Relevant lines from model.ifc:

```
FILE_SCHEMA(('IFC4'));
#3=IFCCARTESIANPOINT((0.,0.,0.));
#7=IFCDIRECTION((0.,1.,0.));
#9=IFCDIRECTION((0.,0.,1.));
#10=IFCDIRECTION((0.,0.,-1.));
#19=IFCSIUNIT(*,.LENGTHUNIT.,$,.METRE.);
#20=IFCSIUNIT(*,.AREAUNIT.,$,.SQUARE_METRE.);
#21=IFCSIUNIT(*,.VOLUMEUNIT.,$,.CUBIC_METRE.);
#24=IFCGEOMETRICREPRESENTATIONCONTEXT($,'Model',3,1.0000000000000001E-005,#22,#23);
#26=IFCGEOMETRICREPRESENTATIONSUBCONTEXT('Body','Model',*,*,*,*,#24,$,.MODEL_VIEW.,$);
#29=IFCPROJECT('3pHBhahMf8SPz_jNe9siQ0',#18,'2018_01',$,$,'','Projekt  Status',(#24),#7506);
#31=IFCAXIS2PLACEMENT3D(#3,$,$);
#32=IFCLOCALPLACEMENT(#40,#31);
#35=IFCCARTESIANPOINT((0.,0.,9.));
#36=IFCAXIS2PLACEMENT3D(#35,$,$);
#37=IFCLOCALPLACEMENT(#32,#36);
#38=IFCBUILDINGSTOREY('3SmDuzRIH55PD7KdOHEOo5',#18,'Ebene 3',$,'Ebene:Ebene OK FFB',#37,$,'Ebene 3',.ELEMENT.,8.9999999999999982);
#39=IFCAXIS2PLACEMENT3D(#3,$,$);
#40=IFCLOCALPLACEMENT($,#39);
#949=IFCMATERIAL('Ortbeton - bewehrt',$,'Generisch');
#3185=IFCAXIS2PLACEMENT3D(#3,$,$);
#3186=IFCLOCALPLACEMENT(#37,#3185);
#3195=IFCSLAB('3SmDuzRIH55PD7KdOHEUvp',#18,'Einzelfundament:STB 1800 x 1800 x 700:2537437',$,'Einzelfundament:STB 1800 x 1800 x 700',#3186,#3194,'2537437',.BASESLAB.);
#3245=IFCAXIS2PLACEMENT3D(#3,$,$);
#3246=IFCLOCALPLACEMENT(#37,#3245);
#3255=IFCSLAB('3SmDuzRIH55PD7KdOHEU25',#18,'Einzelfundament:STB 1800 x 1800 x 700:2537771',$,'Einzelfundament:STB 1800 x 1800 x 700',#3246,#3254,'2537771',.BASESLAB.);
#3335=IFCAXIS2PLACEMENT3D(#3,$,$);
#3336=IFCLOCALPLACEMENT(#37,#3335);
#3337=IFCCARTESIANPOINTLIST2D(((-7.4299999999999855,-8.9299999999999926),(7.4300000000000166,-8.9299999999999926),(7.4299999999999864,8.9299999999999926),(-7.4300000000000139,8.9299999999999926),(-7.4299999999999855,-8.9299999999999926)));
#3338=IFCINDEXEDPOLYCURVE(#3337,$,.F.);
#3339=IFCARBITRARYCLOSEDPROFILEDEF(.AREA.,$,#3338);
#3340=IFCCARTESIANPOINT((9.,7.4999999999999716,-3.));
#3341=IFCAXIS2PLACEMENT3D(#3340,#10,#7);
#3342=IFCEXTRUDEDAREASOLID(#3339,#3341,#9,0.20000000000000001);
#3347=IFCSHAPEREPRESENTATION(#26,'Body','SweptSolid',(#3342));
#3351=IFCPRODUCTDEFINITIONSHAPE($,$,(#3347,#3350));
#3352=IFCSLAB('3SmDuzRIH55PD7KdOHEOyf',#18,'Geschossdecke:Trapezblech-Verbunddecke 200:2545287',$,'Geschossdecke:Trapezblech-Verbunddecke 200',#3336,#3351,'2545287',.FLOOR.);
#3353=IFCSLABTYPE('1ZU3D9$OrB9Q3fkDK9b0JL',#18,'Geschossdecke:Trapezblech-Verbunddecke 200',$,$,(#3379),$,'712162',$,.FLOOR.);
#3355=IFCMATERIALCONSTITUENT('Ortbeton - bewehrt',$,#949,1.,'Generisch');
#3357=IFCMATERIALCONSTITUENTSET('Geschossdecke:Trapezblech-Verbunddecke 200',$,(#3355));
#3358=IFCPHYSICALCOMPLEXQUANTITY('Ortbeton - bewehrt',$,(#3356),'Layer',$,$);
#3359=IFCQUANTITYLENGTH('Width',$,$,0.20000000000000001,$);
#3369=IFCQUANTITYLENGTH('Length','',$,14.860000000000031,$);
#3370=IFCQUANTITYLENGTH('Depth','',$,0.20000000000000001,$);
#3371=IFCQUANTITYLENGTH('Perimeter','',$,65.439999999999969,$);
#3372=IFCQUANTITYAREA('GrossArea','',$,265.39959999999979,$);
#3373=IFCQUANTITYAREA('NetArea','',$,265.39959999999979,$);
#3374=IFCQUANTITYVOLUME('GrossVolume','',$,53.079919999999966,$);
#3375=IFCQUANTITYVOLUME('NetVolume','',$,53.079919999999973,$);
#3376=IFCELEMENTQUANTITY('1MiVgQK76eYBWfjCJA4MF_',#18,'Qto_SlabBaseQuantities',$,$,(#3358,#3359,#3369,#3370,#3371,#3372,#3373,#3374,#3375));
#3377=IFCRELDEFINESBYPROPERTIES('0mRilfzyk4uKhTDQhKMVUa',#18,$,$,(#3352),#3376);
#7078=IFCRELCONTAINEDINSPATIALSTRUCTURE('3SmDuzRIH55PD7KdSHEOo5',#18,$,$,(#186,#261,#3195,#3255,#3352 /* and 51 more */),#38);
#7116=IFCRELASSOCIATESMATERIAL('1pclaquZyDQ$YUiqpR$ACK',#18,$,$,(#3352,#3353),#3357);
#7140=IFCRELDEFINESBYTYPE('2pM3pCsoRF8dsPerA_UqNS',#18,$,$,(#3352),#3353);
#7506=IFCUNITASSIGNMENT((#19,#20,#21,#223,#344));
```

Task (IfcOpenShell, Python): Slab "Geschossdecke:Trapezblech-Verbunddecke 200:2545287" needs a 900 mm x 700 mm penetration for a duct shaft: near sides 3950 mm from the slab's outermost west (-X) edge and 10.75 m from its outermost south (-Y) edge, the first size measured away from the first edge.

```python
import numpy as np
import ifcopenshell
import ifcopenshell.api.feature
import ifcopenshell.api.geometry
import ifcopenshell.api.pset
import ifcopenshell.api.root
import ifcopenshell.geom
import ifcopenshell.util.element
import ifcopenshell.util.placement
import ifcopenshell.util.representation
import ifcopenshell.util.shape
import ifcopenshell.util.unit

model = ifcopenshell.open("model.ifc")
unit_scale = ifcopenshell.util.unit.calculate_unit_scale(model)
area_scale = ifcopenshell.util.unit.calculate_unit_scale(model, "AREAUNIT")
volume_scale = ifcopenshell.util.unit.calculate_unit_scale(model, "VOLUMEUNIT")
settings = ifcopenshell.geom.settings()


def volume(element):
    """Net volume in cubic metres, openings subtracted."""
    shape = ifcopenshell.geom.create_shape(settings, element)
    return ifcopenshell.util.shape.get_volume(shape.geometry)


slab = model.by_guid("3SmDuzRIH55PD7KdOHEOyf")
before = volume(slab)

# Extent in the slab's own axes, in metres. The edges named are its -X and -Y sides.
slab_shape = ifcopenshell.geom.create_shape(settings, slab)
vertices = ifcopenshell.util.shape.get_vertices(slab_shape.geometry)
x_min, y_min, bottom = vertices.min(axis=0)
top = vertices[:, 2].max()

opening = ifcopenshell.api.root.create_entity(model, ifc_class="IfcOpeningElement", name="Duct shaft opening", predefined_type="OPENING")
context = ifcopenshell.util.representation.get_context(model, "Model", "Body", "MODEL_VIEW")
width, depth = 0.9, 0.7
outline = [(0.0, 0.0), (width, 0.0), (width, depth), (0.0, depth), (0.0, 0.0)]
# Overshoot both faces by 50 mm so the cut is clean.
shape = ifcopenshell.api.geometry.add_slab_representation(
    model, context=context, depth=top - bottom + 0.1, polyline=outline
)
ifcopenshell.api.geometry.assign_representation(model, product=opening, representation=shape)

matrix = ifcopenshell.util.placement.get_local_placement(slab.ObjectPlacement)
matrix[:, 3] = matrix @ np.append(np.array([x_min + 3.95, y_min + 10.75, bottom - 0.05]) / unit_scale, 1.0)
ifcopenshell.api.geometry.edit_object_placement(model, product=opening, matrix=matrix, is_si=False)
ifcopenshell.api.feature.add_feature(model, feature=opening, element=slab)

after = volume(slab)

# Update the slab's stored quantities.
qto = model.by_id(ifcopenshell.util.element.get_pset(slab, "Qto_SlabBaseQuantities", should_inherit=False)["id"])
ifcopenshell.api.pset.edit_qto(model, qto=qto, properties={
    "NetArea": after / (top - bottom) / area_scale,
    "NetVolume": after / volume_scale,
})

print(f"slab volume {before:.3f} -> {after:.3f} m3")

model.write("model_rev.ifc")
```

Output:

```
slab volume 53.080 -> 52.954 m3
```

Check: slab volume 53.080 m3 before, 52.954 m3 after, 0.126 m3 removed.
